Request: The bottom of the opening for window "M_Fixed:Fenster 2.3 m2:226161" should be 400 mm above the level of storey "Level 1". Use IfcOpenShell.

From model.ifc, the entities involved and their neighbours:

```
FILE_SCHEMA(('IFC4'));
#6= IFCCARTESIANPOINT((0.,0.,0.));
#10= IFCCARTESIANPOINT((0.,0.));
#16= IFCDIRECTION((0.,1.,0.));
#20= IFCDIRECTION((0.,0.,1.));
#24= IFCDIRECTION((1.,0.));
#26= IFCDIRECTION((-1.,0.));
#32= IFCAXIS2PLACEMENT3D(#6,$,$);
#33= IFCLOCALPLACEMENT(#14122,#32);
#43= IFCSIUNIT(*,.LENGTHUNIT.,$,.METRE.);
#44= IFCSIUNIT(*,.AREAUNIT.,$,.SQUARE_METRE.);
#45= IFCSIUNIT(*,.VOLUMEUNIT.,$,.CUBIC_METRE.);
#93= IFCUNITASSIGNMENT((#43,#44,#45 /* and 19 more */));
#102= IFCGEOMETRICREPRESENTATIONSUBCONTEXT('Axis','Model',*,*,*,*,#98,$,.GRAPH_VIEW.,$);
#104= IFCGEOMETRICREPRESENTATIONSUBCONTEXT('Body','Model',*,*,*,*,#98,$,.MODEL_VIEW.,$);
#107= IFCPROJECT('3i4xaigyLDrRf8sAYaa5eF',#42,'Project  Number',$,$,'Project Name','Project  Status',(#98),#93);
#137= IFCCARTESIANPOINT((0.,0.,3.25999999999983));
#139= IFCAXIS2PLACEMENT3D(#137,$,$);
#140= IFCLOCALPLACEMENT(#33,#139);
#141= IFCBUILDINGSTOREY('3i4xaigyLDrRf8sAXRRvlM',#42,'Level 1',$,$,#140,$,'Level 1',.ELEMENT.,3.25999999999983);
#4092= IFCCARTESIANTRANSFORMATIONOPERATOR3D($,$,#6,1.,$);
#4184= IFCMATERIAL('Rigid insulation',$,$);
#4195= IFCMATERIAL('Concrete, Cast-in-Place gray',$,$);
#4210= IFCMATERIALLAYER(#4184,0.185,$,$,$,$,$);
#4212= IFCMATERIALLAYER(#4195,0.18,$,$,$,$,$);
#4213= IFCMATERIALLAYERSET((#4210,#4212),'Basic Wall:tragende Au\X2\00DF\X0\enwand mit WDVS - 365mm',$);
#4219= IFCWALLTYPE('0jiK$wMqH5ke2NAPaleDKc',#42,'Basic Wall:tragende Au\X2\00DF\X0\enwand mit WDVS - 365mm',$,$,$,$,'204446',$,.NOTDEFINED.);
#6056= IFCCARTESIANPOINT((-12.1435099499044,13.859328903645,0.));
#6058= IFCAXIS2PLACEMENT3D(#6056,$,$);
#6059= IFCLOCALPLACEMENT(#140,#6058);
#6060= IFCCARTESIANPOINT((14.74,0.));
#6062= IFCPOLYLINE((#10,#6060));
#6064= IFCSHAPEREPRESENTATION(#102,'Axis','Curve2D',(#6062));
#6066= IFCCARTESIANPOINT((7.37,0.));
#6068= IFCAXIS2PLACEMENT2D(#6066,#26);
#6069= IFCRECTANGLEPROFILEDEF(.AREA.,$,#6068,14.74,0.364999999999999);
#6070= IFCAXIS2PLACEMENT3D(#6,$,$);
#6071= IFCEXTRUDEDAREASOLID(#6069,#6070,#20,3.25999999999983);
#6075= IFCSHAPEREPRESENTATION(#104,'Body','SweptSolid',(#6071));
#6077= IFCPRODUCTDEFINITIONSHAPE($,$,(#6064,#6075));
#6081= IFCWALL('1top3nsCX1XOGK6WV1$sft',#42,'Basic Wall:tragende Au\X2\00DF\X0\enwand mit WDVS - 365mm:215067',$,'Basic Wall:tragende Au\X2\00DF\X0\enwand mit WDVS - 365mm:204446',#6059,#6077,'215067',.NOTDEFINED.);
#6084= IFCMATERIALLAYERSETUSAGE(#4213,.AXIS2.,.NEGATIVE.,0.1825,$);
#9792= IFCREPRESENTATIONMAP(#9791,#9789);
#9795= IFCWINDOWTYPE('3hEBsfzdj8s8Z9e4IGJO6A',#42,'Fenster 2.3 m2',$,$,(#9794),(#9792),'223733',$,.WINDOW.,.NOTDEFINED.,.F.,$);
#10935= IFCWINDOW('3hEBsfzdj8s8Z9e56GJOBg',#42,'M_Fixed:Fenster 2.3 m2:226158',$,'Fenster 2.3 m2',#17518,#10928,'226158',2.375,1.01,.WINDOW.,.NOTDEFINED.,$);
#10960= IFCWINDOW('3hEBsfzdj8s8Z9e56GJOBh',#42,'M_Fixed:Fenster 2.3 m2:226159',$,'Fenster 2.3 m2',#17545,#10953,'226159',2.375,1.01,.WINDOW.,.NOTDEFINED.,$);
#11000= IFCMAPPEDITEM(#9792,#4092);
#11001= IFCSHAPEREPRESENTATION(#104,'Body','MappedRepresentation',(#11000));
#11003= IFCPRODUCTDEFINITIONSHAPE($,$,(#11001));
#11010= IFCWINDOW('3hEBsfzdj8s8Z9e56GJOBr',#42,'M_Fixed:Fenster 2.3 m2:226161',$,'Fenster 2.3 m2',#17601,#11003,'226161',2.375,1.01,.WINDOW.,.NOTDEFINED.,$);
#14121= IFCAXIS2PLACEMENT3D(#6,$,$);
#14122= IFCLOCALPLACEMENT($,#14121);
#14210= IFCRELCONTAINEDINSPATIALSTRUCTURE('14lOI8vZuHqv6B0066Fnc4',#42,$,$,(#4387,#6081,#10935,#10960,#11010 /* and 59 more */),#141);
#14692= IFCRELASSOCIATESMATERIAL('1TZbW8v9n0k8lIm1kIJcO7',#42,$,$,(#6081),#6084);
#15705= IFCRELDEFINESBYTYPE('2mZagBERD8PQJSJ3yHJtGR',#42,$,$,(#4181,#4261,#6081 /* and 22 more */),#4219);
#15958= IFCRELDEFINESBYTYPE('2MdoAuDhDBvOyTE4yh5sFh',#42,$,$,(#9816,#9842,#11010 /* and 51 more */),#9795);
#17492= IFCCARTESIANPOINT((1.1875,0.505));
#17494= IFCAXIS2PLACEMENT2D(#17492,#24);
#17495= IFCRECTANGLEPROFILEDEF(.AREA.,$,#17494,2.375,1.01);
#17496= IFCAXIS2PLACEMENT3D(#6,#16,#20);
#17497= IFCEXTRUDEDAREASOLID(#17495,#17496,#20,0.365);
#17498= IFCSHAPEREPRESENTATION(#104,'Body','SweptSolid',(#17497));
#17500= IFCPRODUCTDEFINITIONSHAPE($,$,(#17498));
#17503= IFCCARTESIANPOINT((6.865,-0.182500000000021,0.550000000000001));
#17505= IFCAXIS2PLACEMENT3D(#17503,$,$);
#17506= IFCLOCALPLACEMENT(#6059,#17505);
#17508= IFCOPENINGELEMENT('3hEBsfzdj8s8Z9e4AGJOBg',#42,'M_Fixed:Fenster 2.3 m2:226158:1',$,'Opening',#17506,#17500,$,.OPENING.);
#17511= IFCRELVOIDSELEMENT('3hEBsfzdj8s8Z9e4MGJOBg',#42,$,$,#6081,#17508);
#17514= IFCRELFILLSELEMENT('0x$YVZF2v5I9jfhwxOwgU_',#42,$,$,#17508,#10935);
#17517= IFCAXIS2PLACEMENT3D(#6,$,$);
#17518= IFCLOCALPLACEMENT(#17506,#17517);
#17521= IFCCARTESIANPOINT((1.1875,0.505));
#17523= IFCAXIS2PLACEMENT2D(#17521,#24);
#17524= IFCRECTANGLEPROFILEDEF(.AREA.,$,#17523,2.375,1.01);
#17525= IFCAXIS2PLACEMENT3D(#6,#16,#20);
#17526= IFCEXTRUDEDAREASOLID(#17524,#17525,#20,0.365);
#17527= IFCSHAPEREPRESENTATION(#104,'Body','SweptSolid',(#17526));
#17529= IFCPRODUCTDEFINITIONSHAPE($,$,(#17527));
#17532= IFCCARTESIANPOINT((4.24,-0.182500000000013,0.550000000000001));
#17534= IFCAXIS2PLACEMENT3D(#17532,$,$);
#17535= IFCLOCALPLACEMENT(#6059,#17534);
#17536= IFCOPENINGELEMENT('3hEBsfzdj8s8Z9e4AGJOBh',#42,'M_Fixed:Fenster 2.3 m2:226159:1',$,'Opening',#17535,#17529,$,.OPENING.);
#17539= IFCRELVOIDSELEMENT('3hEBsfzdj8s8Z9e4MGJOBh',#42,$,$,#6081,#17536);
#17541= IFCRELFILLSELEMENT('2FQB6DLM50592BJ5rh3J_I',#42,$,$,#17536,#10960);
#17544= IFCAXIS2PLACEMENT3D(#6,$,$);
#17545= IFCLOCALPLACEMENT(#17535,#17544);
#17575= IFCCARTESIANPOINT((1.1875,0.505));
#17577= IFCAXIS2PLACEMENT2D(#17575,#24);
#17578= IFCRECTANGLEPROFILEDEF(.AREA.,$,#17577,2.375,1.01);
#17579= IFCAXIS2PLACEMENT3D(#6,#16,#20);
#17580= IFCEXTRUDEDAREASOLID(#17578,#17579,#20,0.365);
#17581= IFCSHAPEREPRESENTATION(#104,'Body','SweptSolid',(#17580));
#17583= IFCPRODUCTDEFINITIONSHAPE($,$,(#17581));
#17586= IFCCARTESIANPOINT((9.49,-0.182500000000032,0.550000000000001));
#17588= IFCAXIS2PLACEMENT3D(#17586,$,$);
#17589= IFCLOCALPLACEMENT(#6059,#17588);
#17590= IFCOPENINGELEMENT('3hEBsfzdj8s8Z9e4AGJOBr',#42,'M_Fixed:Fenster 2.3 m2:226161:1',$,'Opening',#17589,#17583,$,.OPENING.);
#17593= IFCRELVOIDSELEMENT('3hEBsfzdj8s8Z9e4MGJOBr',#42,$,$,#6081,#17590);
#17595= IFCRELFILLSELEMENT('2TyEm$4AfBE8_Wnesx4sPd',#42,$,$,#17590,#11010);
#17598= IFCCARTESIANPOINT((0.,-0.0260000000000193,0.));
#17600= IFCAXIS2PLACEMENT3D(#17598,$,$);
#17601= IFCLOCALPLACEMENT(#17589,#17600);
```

```python
import numpy as np
import ifcopenshell
import ifcopenshell.api.geometry
import ifcopenshell.geom
import ifcopenshell.util.element
import ifcopenshell.util.placement
import ifcopenshell.util.shape
import ifcopenshell.util.unit

model = ifcopenshell.open("model.ifc")
unit_scale = ifcopenshell.util.unit.calculate_unit_scale(model)

window = model.by_guid("3hEBsfzdj8s8Z9e56GJOBr")
opening = window.FillsVoids[0].RelatingOpeningElement
storey = ifcopenshell.util.element.get_container(window, ifc_class="IfcBuildingStorey")
level = ifcopenshell.util.placement.get_local_placement(storey.ObjectPlacement)[2, 3]

# The opening's origin need not be at the sill, so measure its lowest point.
shape = ifcopenshell.geom.create_shape(ifcopenshell.geom.settings(), opening)
bottom = ifcopenshell.util.shape.get_shape_bottom_elevation(shape, shape.geometry) / unit_scale
dz = level + 0.4 / unit_scale - bottom

shift = np.array([0.0, 0.0, dz])
# The window is placed relative to its opening, so it follows when the opening moves.
matrix = ifcopenshell.util.placement.get_local_placement(opening.ObjectPlacement)
matrix[:3, 3] += shift
ifcopenshell.api.geometry.edit_object_placement(
    model, product=opening, matrix=matrix, is_si=False, should_transform_children=True
)

print(f"moved by {dz * unit_scale:+.3f} m")

model.write("model_v2.ifc")
```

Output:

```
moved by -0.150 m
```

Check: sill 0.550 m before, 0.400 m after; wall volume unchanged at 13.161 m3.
